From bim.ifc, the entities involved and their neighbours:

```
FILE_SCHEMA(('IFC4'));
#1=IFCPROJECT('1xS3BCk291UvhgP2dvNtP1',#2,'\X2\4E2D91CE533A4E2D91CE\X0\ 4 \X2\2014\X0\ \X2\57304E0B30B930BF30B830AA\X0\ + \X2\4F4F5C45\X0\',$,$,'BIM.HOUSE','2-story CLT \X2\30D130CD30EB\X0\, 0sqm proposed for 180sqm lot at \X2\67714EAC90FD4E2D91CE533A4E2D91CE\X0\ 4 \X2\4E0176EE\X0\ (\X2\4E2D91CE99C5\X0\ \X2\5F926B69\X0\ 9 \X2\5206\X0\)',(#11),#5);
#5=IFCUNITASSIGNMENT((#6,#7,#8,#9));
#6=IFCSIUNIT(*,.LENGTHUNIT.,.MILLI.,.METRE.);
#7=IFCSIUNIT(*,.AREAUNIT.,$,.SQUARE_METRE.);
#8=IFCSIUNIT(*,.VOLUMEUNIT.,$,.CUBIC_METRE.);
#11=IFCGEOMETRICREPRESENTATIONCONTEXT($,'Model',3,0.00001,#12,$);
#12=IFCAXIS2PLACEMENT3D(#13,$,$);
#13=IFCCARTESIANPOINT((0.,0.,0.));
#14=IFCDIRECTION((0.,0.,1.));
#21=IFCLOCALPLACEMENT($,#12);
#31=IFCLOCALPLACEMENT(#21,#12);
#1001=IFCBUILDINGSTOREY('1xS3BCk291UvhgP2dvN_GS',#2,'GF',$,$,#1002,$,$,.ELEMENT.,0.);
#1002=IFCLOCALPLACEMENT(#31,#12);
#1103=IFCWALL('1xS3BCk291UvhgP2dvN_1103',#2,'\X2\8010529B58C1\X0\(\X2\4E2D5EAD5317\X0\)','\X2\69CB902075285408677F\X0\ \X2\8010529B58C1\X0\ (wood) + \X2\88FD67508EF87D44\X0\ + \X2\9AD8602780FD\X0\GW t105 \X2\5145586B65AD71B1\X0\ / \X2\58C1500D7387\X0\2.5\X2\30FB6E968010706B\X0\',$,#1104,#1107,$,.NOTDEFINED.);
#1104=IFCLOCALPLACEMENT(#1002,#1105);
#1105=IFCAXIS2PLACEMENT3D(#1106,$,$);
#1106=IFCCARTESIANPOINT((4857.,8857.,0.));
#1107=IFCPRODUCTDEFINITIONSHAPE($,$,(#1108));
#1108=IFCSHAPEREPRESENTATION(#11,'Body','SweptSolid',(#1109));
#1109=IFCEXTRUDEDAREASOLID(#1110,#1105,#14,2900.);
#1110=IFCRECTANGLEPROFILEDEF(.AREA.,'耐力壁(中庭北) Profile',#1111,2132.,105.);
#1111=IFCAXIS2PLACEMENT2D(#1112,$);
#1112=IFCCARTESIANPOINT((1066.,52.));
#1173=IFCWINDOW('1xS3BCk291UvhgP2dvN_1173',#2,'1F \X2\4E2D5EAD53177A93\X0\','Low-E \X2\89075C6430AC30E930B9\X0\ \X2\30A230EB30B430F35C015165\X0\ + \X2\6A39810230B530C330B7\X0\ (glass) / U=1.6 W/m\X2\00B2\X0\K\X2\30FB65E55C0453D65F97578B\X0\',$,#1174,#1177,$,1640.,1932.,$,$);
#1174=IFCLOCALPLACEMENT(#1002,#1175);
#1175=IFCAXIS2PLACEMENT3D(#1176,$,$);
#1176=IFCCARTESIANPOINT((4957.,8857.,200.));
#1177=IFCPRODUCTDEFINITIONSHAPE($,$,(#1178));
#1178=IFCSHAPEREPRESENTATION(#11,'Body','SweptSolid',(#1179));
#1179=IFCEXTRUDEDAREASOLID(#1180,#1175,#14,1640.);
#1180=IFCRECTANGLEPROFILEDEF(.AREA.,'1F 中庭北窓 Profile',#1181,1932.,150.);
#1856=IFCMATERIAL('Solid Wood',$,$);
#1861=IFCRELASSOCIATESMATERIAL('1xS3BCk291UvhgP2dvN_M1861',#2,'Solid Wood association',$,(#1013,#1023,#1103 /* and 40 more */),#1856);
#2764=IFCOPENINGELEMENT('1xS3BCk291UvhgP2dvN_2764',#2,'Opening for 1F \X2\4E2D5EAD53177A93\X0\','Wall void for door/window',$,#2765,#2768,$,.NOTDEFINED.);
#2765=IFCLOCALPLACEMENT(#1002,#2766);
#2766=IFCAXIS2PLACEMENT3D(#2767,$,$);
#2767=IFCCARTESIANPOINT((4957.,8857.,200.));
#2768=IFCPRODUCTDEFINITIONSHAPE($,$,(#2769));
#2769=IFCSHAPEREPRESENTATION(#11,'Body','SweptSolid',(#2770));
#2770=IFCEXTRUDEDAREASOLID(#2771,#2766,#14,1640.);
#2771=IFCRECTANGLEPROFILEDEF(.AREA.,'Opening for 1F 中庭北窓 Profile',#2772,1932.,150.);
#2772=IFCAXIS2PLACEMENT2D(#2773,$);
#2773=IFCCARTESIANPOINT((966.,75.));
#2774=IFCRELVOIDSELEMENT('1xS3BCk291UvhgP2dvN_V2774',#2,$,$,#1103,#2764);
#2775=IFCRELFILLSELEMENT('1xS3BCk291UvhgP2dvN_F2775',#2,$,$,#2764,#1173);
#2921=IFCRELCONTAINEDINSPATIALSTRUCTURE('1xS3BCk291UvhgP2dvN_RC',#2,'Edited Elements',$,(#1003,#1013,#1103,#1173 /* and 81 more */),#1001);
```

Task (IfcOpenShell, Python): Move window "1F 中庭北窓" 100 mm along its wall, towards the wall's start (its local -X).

```python
import ifcopenshell
import ifcopenshell.api.geometry
import ifcopenshell.util.placement

model = ifcopenshell.open("bim.ifc")

window = model.by_guid("1xS3BCk291UvhgP2dvN_1173")
opening = window.FillsVoids[0].RelatingOpeningElement
wall = opening.VoidsElements[0].RelatingBuildingElement

wall_matrix = ifcopenshell.util.placement.get_local_placement(wall.ObjectPlacement)
shift = wall_matrix[:3, 0] * -100.0
before = ifcopenshell.util.placement.get_local_placement(window.ObjectPlacement)[:3, 3].copy()

# The window is not placed relative to its opening, so move both.
for product in (opening, window):
    matrix = ifcopenshell.util.placement.get_local_placement(product.ObjectPlacement)
    matrix[:3, 3] += shift
    ifcopenshell.api.geometry.edit_object_placement(model, product=product, matrix=matrix, is_si=False)

after = ifcopenshell.util.placement.get_local_placement(window.ObjectPlacement)[:3, 3]
print("window moved by", (after - before).round(3) + 0.0)

model.write("bim_edited.ifc")
```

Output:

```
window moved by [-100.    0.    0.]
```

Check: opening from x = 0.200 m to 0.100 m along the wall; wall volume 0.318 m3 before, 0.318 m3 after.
